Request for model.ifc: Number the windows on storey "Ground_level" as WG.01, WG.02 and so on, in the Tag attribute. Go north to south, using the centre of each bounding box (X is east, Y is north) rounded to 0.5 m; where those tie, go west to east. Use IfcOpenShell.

First a look at what the model holds.

```python
import ifcopenshell
import ifcopenshell.util.element
import ifcopenshell.util.placement

model = ifcopenshell.open("model.ifc")
print(model.schema)
storey = next(s for s in model.by_type("IfcBuildingStorey") if s.Name == "Ground_level")
windows = [e for e in ifcopenshell.util.element.get_decomposition(storey) if e.is_a("IfcWindow")]
for e in sorted(windows, key=lambda e: e.id()):
    origin = ifcopenshell.util.placement.get_local_placement(e.ObjectPlacement)[:3, 3]
    print(e.id(), e.Tag, e.Name, origin.round(2) + 0.0, sep=" | ")
```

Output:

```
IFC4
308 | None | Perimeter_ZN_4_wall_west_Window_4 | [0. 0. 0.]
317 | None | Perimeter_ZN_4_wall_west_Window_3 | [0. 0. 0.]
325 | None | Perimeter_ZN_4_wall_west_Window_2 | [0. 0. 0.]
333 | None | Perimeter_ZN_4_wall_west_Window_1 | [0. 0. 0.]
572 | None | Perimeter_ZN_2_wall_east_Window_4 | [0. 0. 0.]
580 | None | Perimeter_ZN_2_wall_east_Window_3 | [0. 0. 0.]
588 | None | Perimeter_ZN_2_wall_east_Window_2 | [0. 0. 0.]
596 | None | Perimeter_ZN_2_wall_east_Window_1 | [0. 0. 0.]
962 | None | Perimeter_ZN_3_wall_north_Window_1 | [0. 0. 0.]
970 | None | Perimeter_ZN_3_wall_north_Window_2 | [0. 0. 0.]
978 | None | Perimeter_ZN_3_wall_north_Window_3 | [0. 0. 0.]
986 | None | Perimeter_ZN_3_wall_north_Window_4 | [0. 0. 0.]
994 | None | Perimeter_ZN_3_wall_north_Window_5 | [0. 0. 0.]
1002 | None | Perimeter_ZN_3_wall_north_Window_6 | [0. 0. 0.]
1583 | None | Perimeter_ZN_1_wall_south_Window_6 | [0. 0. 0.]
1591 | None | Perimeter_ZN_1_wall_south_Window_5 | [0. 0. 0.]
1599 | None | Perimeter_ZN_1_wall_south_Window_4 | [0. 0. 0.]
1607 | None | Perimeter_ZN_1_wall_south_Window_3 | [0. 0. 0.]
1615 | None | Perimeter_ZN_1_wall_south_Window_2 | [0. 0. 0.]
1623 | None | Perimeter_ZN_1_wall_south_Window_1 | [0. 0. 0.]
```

```python
import ifcopenshell
import ifcopenshell.geom
import ifcopenshell.util.element
import ifcopenshell.util.shape

model = ifcopenshell.open("model.ifc")
settings = ifcopenshell.geom.settings()
settings.set("use-world-coords", True)


def centre(element):
    shape = ifcopenshell.geom.create_shape(settings, element)
    return ifcopenshell.util.shape.get_bbox_centroid(shape.geometry)


storey = next(s for s in model.by_type("IfcBuildingStorey") if s.Name == "Ground_level")
windows = [e for e in ifcopenshell.util.element.get_decomposition(storey) if e.is_a("IfcWindow")]

# Insertion points can sit at a corner or the storey origin, so sort by the geometry (in metres).
centres = {e: centre(e) for e in windows}
windows.sort(key=lambda e: (-round(centres[e][1] / 0.5), centres[e][0]))

for i, e in enumerate(windows, start=1):
    number = f"WG.{i:02d}"
    e.Tag = number
    print(e.id(), number)

model.write("model-out.ifc")
```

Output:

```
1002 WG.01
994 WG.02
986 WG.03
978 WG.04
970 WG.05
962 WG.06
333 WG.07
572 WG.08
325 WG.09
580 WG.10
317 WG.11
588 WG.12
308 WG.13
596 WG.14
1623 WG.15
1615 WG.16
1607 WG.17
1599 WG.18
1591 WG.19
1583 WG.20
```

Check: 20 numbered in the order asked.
